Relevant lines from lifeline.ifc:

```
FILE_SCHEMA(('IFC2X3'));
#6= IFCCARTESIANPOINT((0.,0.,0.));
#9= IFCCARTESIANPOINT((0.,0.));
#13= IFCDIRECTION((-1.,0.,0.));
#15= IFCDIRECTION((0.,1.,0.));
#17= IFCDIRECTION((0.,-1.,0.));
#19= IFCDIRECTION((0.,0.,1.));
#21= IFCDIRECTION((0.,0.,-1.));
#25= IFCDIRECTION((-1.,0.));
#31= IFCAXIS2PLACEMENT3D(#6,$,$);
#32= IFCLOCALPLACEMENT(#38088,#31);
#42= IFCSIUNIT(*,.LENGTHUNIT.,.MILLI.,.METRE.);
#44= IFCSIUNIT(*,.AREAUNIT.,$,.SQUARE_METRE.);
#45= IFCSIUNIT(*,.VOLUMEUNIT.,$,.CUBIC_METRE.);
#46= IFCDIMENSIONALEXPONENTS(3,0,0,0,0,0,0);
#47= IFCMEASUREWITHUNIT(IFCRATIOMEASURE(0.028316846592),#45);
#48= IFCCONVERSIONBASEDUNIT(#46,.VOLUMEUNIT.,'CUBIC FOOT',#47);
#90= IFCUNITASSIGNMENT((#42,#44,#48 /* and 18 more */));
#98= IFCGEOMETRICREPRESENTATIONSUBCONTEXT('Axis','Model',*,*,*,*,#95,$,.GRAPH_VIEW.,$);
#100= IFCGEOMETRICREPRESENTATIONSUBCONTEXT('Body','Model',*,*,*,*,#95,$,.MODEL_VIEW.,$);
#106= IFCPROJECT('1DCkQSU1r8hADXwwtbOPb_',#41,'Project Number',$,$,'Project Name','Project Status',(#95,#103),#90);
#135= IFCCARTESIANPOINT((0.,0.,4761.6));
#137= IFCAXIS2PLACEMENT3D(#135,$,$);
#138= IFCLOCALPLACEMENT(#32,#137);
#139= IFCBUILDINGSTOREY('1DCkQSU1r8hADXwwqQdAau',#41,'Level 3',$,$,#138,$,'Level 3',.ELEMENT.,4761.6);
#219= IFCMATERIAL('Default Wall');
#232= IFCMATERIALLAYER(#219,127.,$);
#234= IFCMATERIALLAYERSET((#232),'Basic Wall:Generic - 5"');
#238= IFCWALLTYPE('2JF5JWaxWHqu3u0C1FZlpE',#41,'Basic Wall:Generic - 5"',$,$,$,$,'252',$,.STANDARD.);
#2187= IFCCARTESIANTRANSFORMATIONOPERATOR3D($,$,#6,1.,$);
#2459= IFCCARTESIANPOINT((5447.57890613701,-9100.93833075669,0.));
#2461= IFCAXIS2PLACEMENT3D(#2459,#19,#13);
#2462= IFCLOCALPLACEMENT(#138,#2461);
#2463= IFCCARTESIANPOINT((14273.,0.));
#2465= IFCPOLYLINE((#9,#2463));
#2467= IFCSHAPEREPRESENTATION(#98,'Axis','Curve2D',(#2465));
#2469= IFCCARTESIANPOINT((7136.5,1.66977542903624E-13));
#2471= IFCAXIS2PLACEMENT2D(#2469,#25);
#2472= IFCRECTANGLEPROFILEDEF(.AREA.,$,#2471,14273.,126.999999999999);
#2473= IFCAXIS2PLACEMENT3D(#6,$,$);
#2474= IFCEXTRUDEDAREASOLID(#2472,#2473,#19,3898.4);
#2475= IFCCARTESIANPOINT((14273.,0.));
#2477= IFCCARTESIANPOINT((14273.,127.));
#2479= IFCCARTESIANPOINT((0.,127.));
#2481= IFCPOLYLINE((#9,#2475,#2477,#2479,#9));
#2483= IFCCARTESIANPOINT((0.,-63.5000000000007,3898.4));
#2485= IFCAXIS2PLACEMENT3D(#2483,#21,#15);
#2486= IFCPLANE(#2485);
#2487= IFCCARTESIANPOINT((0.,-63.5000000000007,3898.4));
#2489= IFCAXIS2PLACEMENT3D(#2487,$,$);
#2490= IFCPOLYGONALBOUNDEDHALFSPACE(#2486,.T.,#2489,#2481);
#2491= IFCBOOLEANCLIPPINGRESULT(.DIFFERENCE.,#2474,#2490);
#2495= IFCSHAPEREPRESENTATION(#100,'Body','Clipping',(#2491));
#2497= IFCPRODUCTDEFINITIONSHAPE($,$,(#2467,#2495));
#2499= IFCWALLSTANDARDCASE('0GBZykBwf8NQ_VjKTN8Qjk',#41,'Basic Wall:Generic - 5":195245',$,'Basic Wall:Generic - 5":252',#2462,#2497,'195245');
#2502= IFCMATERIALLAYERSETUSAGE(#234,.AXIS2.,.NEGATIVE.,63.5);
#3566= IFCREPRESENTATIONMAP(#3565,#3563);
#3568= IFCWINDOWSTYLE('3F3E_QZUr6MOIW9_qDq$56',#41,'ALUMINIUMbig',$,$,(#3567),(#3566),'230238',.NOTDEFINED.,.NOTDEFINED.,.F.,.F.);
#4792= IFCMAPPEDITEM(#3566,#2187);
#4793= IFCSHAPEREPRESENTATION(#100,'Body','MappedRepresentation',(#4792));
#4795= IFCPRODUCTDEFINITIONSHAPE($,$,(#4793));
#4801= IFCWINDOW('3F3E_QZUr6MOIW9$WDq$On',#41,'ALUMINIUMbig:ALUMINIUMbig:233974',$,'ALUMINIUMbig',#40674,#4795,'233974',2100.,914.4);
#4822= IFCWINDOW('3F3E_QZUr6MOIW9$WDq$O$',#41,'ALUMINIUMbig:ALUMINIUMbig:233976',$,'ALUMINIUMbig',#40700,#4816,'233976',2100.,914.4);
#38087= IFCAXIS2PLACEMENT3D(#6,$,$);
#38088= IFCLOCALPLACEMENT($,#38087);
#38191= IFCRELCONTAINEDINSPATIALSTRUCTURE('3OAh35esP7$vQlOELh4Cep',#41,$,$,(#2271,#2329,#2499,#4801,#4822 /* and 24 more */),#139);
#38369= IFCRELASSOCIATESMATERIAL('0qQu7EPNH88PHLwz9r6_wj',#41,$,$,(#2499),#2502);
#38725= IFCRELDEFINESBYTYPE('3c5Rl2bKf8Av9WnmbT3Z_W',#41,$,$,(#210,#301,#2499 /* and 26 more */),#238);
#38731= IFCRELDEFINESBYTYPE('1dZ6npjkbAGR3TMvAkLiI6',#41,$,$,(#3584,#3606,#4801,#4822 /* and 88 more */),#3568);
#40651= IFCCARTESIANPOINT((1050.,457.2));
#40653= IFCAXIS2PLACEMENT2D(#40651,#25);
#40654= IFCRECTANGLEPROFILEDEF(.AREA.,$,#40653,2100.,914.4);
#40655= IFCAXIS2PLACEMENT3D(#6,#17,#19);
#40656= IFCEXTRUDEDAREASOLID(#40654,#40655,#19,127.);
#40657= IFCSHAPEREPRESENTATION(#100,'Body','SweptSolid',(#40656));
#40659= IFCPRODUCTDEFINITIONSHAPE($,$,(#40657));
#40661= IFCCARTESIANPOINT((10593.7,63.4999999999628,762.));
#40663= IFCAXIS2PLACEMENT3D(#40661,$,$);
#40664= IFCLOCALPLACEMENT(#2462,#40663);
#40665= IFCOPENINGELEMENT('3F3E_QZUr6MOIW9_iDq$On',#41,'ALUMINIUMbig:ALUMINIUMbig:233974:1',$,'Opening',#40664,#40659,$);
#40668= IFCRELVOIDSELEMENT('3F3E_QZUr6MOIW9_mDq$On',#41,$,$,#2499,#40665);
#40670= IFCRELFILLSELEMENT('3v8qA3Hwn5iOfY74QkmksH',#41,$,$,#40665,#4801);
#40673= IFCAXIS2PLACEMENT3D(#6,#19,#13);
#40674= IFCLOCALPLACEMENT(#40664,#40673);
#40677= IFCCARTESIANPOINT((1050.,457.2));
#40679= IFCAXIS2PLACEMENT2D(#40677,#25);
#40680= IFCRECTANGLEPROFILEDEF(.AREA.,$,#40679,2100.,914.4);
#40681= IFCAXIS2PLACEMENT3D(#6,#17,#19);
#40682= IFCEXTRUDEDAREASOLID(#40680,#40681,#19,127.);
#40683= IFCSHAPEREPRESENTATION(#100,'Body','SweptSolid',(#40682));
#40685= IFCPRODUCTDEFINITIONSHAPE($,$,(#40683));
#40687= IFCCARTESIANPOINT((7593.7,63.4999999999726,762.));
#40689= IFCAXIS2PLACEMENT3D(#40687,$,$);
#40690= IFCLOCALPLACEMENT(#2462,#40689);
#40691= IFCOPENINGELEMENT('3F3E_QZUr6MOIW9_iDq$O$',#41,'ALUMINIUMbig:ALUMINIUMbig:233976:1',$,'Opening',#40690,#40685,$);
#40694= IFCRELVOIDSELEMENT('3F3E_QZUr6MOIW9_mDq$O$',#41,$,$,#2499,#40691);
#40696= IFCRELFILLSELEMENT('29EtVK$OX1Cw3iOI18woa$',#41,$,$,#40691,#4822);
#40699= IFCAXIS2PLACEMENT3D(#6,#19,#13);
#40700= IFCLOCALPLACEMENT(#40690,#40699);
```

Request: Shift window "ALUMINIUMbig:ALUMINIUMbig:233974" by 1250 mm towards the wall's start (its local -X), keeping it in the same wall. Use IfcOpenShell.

```python
import ifcopenshell
import ifcopenshell.api.geometry
import ifcopenshell.util.placement

model = ifcopenshell.open("lifeline.ifc")

window = model.by_guid("3F3E_QZUr6MOIW9$WDq$On")
opening = window.FillsVoids[0].RelatingOpeningElement
wall = opening.VoidsElements[0].RelatingBuildingElement

wall_matrix = ifcopenshell.util.placement.get_local_placement(wall.ObjectPlacement)
shift = wall_matrix[:3, 0] * -1250.0
before = ifcopenshell.util.placement.get_local_placement(window.ObjectPlacement)[:3, 3].copy()

# The window is placed relative to its opening, so it follows when the opening moves.
matrix = ifcopenshell.util.placement.get_local_placement(opening.ObjectPlacement)
matrix[:3, 3] += shift
ifcopenshell.api.geometry.edit_object_placement(
    model, product=opening, matrix=matrix, is_si=False, should_transform_children=True
)

after = ifcopenshell.util.placement.get_local_placement(window.ObjectPlacement)[:3, 3]
print("window moved by", (after - before).round(3) + 0.0)

model.write("lifeline_rev.ifc")
```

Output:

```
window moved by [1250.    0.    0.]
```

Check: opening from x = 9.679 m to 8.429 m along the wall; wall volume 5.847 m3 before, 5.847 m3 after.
